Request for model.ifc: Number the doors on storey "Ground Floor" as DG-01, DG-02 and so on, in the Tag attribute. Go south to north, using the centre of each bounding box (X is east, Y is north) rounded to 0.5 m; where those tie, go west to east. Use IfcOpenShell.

First a look at what the model holds.

```python
import ifcopenshell
import ifcopenshell.util.element
import ifcopenshell.util.placement

model = ifcopenshell.open("model.ifc")
print(model.schema)
storey = next(s for s in model.by_type("IfcBuildingStorey") if s.Name == "Ground Floor")
doors = [e for e in ifcopenshell.util.element.get_decomposition(storey) if e.is_a("IfcDoor")]
for e in sorted(doors, key=lambda e: e.id()):
    origin = ifcopenshell.util.placement.get_local_placement(e.ObjectPlacement)[:3, 3]
    print(e.id(), e.Tag, e.Name, origin.round(2) + 0.0, sep=" | ")
```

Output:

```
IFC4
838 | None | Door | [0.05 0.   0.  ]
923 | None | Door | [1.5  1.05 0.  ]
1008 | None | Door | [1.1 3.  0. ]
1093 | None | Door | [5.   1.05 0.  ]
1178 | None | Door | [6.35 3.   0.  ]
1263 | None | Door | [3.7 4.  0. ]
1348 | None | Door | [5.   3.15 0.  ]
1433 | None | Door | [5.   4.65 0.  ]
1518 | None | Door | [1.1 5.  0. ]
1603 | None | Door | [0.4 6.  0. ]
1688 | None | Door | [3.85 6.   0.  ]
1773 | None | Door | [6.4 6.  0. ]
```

```python
import ifcopenshell
import ifcopenshell.geom
import ifcopenshell.util.element
import ifcopenshell.util.shape

model = ifcopenshell.open("model.ifc")
settings = ifcopenshell.geom.settings()
settings.set("use-world-coords", True)


def centre(element):
    shape = ifcopenshell.geom.create_shape(settings, element)
    return ifcopenshell.util.shape.get_bbox_centroid(shape.geometry)


storey = next(s for s in model.by_type("IfcBuildingStorey") if s.Name == "Ground Floor")
doors = [e for e in ifcopenshell.util.element.get_decomposition(storey) if e.is_a("IfcDoor")]

# Insertion points can sit at a corner or the storey origin, so sort by the geometry (in metres).
centres = {e: centre(e) for e in doors}
doors.sort(key=lambda e: (round(centres[e][1] / 0.5), centres[e][0]))

for i, e in enumerate(doors, start=1):
    number = f"DG-{i:02d}"
    e.Tag = number
    print(e.id(), number)

model.write("model_updated.ifc")
```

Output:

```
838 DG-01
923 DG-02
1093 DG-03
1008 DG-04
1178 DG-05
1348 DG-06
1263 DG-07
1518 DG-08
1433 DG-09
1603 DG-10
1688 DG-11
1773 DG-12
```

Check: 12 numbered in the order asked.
